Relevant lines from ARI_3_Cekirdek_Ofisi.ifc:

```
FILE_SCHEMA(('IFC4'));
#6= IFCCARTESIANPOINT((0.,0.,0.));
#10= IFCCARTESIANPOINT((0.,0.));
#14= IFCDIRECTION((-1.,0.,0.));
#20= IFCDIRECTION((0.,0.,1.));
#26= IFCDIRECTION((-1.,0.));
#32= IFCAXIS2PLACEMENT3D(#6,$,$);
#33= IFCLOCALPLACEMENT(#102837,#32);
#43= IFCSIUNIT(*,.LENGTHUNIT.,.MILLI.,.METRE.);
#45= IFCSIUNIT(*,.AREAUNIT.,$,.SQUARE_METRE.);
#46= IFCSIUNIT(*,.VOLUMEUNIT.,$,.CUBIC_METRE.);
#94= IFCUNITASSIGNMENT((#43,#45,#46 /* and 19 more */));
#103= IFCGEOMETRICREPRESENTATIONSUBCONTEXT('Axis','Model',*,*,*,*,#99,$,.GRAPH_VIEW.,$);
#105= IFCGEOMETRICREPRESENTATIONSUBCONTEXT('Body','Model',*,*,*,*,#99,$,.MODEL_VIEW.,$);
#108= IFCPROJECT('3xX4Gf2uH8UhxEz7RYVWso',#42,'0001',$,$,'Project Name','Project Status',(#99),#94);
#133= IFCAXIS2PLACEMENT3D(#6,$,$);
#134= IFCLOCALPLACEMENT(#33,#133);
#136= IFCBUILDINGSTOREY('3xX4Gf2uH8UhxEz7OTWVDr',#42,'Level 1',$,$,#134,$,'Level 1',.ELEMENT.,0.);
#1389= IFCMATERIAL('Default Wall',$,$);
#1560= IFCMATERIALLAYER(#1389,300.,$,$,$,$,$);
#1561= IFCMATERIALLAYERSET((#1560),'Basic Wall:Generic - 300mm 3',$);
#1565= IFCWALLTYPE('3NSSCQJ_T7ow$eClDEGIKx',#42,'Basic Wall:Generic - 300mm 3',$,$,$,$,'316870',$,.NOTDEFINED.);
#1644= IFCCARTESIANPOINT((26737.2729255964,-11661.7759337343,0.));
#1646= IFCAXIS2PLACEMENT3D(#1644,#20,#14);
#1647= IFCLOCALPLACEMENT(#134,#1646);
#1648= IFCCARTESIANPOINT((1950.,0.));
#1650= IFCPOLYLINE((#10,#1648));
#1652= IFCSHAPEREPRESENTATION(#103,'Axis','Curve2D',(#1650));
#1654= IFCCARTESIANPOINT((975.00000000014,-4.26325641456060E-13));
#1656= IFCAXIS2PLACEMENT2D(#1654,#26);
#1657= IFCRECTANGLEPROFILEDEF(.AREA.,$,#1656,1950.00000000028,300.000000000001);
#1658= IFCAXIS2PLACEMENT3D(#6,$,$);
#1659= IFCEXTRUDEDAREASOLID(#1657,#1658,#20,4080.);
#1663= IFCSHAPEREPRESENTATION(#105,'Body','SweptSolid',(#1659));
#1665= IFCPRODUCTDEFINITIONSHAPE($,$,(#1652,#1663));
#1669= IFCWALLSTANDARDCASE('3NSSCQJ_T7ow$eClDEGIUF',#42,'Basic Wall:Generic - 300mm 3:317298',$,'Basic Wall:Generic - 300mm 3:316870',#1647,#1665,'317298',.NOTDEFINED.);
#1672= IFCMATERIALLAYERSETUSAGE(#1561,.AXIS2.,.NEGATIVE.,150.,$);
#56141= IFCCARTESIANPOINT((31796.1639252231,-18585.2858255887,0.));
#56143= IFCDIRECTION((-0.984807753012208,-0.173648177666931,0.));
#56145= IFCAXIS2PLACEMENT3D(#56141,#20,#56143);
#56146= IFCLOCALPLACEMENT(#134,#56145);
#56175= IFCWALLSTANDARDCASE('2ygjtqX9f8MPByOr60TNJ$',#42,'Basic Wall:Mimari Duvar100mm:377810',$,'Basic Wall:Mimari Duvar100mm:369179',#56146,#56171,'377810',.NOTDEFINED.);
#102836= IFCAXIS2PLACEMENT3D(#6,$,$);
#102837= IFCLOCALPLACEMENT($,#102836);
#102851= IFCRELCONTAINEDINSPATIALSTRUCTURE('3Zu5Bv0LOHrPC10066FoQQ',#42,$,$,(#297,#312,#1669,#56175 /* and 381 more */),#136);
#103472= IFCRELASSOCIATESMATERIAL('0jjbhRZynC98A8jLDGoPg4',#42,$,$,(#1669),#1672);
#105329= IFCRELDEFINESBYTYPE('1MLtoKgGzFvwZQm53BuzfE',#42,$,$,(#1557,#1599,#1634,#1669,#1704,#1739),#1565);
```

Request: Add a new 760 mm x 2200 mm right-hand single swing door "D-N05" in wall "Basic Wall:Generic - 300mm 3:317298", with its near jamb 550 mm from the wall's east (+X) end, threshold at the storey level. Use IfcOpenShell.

```python
import numpy as np
import ifcopenshell
import ifcopenshell.api.feature
import ifcopenshell.api.geometry
import ifcopenshell.api.root
import ifcopenshell.api.spatial
import ifcopenshell.geom
import ifcopenshell.util.element
import ifcopenshell.util.placement
import ifcopenshell.util.representation
import ifcopenshell.util.shape
import ifcopenshell.util.unit

model = ifcopenshell.open("ARI_3_Cekirdek_Ofisi.ifc")
unit_scale = ifcopenshell.util.unit.calculate_unit_scale(model)
settings = ifcopenshell.geom.settings()


def volume(element):
    """Net volume in cubic metres, openings subtracted."""
    shape = ifcopenshell.geom.create_shape(settings, element)
    return ifcopenshell.util.shape.get_volume(shape.geometry)


wall = model.by_guid("3NSSCQJ_T7ow$eClDEGIUF")
storey = ifcopenshell.util.element.get_container(wall, ifc_class="IfcBuildingStorey")
context = ifcopenshell.util.representation.get_context(model, "Model", "Body", "MODEL_VIEW")
before = volume(wall)

width, height, from_end, sill = 0.76, 2.2, 0.55, 0.0  # metres

# The wall runs along its own X axis, and the end named is its -X end.
wall_shape = ifcopenshell.geom.create_shape(settings, wall)
x, y, z = ifcopenshell.util.shape.get_vertices(wall_shape.geometry).T
start = x.min() + from_end
face, thickness = float(y.min()), float(y.max() - y.min())
wall_matrix = ifcopenshell.util.placement.get_local_placement(wall.ObjectPlacement)
level = ifcopenshell.util.placement.get_local_placement(storey.ObjectPlacement)[2, 3]


def in_wall(x, y):
    """Placement at x, y metres in the wall's axes, at sill height."""
    matrix = wall_matrix.copy()
    matrix[:, 3] = wall_matrix @ np.array([x / unit_scale, y / unit_scale, 0.0, 1.0])
    matrix[2, 3] = level + sill / unit_scale
    return matrix


# Opening: a box that overshoots both wall faces by 50 mm.
opening = ifcopenshell.api.root.create_entity(model, ifc_class="IfcOpeningElement", predefined_type="OPENING")
box = ifcopenshell.api.geometry.add_wall_representation(
    model, context=context, length=width, height=height, thickness=thickness + 0.1
)
ifcopenshell.api.geometry.assign_representation(model, product=opening, representation=box)
ifcopenshell.api.geometry.edit_object_placement(model, product=opening, matrix=in_wall(start, face - 0.05), is_si=False)
ifcopenshell.api.feature.add_feature(model, feature=opening, element=wall)

door = ifcopenshell.api.root.create_entity(model, ifc_class="IfcDoor", name="D-N05", predefined_type="DOOR")
door.OverallWidth, door.OverallHeight = width / unit_scale, height / unit_scale
door.OperationType = "SINGLE_SWING_RIGHT"
body = ifcopenshell.api.geometry.add_door_representation(
    model,
    context=context,
    overall_width=door.OverallWidth,
    overall_height=door.OverallHeight,
    operation_type="SINGLE_SWING_RIGHT",
    lining_properties={"LiningDepth": thickness / unit_scale, "ThresholdDepth": thickness / unit_scale},
)
ifcopenshell.api.geometry.assign_representation(model, product=door, representation=body)
ifcopenshell.api.spatial.assign_container(model, products=[door], relating_structure=storey)
ifcopenshell.api.feature.add_filling(model, opening=opening, element=door)

# The lining spans the wall, so the door starts at the wall face.
ifcopenshell.api.geometry.edit_object_placement(model, product=door, matrix=in_wall(start, face), is_si=False)

after = volume(wall)

print(f"wall volume {before:.3f} -> {after:.3f} m3")

model.write("ARI_3_Cekirdek_Ofisi_v2.ifc")
```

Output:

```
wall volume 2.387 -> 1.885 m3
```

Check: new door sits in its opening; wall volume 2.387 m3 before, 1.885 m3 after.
